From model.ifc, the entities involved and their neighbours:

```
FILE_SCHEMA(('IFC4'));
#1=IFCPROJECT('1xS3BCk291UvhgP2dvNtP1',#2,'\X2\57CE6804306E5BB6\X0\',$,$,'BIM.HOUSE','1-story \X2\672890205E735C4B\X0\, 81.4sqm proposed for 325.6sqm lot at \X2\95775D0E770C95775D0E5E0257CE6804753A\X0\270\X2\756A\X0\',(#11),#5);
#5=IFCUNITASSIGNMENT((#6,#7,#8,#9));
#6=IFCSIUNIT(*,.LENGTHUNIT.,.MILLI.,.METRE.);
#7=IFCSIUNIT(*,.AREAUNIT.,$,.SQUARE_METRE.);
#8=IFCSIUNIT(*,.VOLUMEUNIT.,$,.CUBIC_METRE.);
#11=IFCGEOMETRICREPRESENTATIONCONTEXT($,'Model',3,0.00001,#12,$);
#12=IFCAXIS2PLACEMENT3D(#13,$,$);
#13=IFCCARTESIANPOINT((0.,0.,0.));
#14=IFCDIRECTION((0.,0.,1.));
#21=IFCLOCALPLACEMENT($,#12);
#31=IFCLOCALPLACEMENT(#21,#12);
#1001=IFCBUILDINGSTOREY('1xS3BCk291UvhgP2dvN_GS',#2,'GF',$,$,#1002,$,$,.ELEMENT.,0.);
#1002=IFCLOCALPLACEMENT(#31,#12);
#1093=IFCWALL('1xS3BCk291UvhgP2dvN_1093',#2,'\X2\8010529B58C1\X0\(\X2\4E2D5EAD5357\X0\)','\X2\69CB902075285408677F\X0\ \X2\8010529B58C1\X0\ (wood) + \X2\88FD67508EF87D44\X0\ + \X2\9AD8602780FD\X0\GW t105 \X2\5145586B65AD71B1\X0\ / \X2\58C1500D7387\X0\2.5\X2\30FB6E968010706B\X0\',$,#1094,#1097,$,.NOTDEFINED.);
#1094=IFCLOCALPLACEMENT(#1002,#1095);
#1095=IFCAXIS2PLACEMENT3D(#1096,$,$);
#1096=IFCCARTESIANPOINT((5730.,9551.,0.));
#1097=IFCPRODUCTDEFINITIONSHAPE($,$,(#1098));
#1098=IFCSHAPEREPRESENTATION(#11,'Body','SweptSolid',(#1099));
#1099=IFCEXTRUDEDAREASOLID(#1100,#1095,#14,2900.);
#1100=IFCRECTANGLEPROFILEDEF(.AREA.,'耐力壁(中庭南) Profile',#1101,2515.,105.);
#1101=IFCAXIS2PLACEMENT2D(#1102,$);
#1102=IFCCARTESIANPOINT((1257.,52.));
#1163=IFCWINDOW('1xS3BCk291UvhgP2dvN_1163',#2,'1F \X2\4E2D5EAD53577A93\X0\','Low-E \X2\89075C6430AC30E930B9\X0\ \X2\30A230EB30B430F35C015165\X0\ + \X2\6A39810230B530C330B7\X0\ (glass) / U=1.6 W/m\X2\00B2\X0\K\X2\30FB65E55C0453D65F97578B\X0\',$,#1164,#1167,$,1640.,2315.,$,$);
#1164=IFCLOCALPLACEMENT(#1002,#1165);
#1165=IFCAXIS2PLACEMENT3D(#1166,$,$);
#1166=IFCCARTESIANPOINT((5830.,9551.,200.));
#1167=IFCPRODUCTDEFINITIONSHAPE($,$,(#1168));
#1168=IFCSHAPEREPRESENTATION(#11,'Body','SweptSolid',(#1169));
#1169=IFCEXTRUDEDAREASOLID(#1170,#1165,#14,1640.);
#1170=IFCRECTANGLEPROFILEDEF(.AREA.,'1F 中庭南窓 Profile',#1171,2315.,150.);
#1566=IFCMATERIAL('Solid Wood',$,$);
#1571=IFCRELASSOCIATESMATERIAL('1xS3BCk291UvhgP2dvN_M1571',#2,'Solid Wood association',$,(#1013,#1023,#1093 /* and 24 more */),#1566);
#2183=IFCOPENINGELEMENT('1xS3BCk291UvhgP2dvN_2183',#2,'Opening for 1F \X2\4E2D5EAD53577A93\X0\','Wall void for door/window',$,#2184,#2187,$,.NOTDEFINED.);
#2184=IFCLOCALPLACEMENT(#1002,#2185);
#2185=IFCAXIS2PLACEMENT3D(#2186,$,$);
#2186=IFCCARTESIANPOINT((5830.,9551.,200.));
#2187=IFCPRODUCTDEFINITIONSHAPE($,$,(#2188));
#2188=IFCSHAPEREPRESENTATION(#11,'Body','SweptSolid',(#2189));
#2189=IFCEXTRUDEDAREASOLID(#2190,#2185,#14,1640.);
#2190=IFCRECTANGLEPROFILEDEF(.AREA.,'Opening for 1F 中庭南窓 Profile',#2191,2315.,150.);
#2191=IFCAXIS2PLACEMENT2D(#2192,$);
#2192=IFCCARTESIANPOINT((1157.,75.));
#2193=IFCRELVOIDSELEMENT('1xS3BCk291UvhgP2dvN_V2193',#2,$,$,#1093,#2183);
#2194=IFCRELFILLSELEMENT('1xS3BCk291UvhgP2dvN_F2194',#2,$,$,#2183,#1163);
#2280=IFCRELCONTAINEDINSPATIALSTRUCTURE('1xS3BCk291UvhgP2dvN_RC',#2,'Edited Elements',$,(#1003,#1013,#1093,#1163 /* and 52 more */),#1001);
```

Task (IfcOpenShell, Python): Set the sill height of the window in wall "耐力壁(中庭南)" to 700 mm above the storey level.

```python
import numpy as np
import ifcopenshell
import ifcopenshell.api.geometry
import ifcopenshell.geom
import ifcopenshell.util.element
import ifcopenshell.util.placement
import ifcopenshell.util.shape
import ifcopenshell.util.unit

model = ifcopenshell.open("model.ifc")
unit_scale = ifcopenshell.util.unit.calculate_unit_scale(model)

window = model.by_id(1163)
opening = window.FillsVoids[0].RelatingOpeningElement
storey = ifcopenshell.util.element.get_container(window, ifc_class="IfcBuildingStorey")
level = ifcopenshell.util.placement.get_local_placement(storey.ObjectPlacement)[2, 3]

# The opening's origin need not be at the sill, so measure its lowest point.
shape = ifcopenshell.geom.create_shape(ifcopenshell.geom.settings(), opening)
bottom = ifcopenshell.util.shape.get_shape_bottom_elevation(shape, shape.geometry) / unit_scale
dz = level + 0.7 / unit_scale - bottom

shift = np.array([0.0, 0.0, dz])
# The window is not placed relative to its opening, so move both.
for product in (opening, window):
    matrix = ifcopenshell.util.placement.get_local_placement(product.ObjectPlacement)
    matrix[:3, 3] += shift
    ifcopenshell.api.geometry.edit_object_placement(model, product=product, matrix=matrix, is_si=False)

print(f"moved by {dz * unit_scale:+.3f} m")

model.write("model_edited.ifc")
```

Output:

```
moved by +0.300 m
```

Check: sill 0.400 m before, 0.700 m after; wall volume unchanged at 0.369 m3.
